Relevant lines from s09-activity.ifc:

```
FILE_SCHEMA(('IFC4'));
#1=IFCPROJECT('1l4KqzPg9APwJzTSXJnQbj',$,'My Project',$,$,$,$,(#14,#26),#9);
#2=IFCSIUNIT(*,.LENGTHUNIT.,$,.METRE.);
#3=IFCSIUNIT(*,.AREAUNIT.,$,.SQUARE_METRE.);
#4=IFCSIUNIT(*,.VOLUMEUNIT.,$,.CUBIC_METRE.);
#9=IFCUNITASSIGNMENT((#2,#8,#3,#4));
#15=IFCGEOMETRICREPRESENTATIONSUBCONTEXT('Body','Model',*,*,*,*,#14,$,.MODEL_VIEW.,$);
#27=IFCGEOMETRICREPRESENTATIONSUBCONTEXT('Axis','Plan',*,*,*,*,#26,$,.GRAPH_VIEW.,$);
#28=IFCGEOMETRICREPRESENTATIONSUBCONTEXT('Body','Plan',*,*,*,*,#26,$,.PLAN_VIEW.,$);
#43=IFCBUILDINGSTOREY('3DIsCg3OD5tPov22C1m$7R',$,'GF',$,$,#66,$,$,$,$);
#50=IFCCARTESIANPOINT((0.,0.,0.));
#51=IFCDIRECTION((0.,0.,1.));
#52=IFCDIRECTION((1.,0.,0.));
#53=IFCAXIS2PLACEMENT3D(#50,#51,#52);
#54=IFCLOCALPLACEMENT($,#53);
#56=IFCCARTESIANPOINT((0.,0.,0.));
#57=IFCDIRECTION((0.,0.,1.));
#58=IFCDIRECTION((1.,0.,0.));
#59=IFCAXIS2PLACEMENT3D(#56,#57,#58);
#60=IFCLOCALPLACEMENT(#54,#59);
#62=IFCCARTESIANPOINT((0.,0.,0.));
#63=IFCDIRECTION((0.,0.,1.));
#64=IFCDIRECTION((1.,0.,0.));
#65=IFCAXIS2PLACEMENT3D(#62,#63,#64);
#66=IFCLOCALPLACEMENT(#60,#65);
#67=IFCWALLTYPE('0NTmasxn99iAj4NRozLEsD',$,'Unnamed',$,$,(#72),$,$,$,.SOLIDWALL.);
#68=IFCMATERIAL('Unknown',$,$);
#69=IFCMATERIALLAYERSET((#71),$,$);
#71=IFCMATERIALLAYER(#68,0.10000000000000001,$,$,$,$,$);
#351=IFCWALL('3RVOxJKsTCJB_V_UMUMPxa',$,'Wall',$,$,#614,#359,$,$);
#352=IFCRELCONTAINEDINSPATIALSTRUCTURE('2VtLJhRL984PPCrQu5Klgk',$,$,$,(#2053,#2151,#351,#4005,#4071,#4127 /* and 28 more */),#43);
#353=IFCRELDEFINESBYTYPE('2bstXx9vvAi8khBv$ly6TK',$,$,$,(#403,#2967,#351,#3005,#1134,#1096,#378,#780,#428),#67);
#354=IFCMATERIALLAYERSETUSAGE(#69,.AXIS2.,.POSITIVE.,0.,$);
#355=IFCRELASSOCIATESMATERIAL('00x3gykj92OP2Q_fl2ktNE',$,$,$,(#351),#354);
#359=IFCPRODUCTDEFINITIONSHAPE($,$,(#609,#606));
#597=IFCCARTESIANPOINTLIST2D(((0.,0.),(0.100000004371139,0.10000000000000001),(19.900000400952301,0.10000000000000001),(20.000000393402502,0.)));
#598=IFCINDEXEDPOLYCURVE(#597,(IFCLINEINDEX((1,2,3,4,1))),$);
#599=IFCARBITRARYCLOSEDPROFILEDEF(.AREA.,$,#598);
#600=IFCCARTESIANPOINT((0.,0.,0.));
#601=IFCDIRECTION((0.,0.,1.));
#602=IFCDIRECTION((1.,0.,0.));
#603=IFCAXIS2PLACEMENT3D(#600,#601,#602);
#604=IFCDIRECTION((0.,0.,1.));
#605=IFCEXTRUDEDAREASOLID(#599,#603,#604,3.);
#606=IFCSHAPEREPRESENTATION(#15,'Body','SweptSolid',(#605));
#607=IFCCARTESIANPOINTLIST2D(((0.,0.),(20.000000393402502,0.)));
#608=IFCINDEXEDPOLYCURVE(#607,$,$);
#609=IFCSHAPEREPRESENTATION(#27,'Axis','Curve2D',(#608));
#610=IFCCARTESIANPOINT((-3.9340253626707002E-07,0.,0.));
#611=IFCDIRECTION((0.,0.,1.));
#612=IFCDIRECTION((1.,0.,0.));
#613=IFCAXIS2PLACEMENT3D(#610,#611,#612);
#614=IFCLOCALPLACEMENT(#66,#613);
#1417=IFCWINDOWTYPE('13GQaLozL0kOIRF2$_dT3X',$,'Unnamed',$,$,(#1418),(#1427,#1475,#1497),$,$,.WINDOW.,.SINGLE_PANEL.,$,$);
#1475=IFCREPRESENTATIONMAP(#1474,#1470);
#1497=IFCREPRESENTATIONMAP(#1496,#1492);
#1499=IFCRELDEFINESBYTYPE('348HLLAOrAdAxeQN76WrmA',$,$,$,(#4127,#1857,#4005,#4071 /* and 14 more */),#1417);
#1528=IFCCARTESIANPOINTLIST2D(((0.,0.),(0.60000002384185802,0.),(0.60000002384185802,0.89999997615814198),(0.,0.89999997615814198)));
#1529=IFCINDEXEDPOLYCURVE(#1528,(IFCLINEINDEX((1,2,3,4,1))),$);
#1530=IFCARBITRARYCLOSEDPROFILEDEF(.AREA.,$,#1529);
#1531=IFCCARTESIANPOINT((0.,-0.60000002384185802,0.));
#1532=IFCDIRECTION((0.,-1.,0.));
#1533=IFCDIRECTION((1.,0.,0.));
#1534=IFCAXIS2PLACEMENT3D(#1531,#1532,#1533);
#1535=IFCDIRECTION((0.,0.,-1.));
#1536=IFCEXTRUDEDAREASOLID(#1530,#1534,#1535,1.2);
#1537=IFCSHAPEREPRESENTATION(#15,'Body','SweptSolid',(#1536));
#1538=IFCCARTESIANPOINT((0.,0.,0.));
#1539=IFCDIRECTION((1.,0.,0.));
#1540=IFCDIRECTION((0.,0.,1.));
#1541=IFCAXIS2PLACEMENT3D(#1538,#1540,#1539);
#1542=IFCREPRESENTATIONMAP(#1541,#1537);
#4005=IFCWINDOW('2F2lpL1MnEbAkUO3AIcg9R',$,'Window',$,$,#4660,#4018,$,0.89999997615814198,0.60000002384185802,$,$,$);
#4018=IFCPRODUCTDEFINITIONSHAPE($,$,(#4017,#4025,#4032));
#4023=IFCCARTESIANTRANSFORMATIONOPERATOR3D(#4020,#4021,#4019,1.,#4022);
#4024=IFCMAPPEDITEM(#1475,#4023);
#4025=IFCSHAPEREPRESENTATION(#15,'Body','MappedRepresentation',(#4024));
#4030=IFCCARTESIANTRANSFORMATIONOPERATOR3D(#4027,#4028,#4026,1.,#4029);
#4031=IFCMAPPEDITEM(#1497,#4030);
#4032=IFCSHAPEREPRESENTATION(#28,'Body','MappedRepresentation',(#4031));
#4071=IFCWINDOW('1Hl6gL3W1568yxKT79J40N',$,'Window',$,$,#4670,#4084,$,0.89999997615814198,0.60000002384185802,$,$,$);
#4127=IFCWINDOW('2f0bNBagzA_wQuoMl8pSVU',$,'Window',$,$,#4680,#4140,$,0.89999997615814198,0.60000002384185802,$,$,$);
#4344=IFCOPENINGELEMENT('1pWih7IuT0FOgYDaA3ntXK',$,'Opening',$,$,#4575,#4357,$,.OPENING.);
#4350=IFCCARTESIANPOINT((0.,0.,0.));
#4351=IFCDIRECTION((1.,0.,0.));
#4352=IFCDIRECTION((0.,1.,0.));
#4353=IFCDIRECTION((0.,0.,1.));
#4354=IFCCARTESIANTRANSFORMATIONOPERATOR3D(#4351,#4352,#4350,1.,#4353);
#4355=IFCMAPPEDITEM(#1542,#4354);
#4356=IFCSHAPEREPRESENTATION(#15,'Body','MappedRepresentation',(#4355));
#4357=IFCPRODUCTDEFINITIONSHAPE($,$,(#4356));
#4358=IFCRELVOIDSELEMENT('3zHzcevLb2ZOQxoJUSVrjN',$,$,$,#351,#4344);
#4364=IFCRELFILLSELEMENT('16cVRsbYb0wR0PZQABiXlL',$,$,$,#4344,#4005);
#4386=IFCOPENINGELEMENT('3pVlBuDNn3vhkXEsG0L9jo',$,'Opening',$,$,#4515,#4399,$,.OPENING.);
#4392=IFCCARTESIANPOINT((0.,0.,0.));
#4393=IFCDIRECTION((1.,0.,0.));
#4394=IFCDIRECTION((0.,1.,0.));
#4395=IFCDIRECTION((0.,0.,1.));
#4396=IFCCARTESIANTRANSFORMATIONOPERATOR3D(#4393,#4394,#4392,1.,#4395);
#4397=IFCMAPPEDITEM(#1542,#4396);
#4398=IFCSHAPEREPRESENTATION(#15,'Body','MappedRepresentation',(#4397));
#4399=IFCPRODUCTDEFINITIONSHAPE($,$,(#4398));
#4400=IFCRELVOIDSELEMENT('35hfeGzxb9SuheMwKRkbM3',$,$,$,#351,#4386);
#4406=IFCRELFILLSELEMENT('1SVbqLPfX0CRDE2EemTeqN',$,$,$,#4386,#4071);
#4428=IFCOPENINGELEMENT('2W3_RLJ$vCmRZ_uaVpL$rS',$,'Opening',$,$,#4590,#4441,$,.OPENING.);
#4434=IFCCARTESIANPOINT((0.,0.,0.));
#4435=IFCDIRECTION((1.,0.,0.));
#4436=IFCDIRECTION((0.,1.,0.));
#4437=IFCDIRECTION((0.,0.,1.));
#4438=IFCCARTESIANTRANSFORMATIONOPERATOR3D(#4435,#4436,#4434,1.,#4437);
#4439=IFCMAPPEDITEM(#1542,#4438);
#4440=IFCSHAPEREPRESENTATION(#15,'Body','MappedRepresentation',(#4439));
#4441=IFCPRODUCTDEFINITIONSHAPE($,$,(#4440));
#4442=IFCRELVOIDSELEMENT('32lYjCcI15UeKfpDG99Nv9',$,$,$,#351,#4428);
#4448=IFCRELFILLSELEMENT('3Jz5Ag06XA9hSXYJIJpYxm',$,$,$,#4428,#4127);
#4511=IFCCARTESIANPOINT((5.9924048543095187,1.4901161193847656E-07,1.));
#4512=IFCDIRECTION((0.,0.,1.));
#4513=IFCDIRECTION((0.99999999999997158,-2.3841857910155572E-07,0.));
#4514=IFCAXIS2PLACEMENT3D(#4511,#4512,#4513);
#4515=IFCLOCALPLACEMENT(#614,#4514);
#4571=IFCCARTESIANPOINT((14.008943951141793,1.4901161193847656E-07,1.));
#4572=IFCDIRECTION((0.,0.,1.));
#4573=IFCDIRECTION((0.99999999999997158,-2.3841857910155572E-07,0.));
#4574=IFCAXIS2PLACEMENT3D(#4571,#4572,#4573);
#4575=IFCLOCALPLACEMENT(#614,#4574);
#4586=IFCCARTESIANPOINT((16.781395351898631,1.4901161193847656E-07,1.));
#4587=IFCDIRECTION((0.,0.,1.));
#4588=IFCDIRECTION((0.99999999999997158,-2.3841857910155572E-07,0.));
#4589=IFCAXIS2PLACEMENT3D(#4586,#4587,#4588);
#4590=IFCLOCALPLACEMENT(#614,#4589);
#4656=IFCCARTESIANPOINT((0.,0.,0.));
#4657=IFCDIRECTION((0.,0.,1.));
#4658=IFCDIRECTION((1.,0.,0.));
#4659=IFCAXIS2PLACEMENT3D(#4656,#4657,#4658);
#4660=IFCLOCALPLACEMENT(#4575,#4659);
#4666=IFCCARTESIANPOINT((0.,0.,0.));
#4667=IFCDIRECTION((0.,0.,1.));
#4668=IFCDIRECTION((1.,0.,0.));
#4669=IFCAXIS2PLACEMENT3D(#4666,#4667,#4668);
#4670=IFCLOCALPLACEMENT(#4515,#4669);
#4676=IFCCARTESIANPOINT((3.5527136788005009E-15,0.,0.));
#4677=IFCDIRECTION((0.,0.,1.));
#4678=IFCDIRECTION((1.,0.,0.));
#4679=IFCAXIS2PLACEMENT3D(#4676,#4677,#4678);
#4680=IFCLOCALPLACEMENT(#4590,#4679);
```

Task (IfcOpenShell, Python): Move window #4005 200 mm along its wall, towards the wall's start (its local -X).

```python
import ifcopenshell
import ifcopenshell.api.geometry
import ifcopenshell.util.placement

model = ifcopenshell.open("s09-activity.ifc")

window = model.by_guid("2F2lpL1MnEbAkUO3AIcg9R")
opening = window.FillsVoids[0].RelatingOpeningElement
wall = opening.VoidsElements[0].RelatingBuildingElement

wall_matrix = ifcopenshell.util.placement.get_local_placement(wall.ObjectPlacement)
shift = wall_matrix[:3, 0] * -0.2
before = ifcopenshell.util.placement.get_local_placement(window.ObjectPlacement)[:3, 3].copy()

# The window is placed relative to its opening, so it follows when the opening moves.
matrix = ifcopenshell.util.placement.get_local_placement(opening.ObjectPlacement)
matrix[:3, 3] += shift
ifcopenshell.api.geometry.edit_object_placement(
    model, product=opening, matrix=matrix, is_si=False, should_transform_children=True
)

after = ifcopenshell.util.placement.get_local_placement(window.ObjectPlacement)[:3, 3]
print("window moved by", (after - before).round(3) + 0.0)

model.write("s09-activity_v2.ifc")
```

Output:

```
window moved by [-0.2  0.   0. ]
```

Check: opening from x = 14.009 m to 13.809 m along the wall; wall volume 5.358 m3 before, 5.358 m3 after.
